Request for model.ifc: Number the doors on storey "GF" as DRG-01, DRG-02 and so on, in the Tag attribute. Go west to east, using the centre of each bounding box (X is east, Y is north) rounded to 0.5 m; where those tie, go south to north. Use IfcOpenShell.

First a look at what the model holds.

```python
import ifcopenshell
import ifcopenshell.util.element
import ifcopenshell.util.placement

model = ifcopenshell.open("model.ifc")
print(model.schema)
storey = next(s for s in model.by_type("IfcBuildingStorey") if s.Name == "GF")
doors = [e for e in ifcopenshell.util.element.get_decomposition(storey) if e.is_a("IfcDoor")]
for e in sorted(doors, key=lambda e: e.id()):
    origin = ifcopenshell.util.placement.get_local_placement(e.ObjectPlacement)[:3, 3]
    print(e.id(), e.Tag, e.Name, origin.round(2) + 0.0, sep=" | ")
```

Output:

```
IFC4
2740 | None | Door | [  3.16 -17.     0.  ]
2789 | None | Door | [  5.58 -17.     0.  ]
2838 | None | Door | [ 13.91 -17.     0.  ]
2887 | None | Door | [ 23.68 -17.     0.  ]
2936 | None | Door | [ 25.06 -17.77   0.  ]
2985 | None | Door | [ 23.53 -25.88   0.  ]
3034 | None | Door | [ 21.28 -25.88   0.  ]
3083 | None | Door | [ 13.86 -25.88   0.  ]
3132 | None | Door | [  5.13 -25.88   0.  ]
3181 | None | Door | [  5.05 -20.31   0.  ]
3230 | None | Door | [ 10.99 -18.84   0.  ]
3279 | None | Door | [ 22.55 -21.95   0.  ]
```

```python
import ifcopenshell
import ifcopenshell.geom
import ifcopenshell.util.element
import ifcopenshell.util.shape

model = ifcopenshell.open("model.ifc")
settings = ifcopenshell.geom.settings()
settings.set("use-world-coords", True)


def centre(element):
    shape = ifcopenshell.geom.create_shape(settings, element)
    return ifcopenshell.util.shape.get_bbox_centroid(shape.geometry)


storey = next(s for s in model.by_type("IfcBuildingStorey") if s.Name == "GF")
doors = [e for e in ifcopenshell.util.element.get_decomposition(storey) if e.is_a("IfcDoor")]

# Insertion points can sit at a corner or the storey origin, so sort by the geometry (in metres).
centres = {e: centre(e) for e in doors}
doors.sort(key=lambda e: (round(centres[e][0] / 0.5), centres[e][1]))

for i, e in enumerate(doors, start=1):
    number = f"DRG-{i:02d}"
    e.Tag = number
    print(e.id(), number)

model.write("model-out.ifc")
```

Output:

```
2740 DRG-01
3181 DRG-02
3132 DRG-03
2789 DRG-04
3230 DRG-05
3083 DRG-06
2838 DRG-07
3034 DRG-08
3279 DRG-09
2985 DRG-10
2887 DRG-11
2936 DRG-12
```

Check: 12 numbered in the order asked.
